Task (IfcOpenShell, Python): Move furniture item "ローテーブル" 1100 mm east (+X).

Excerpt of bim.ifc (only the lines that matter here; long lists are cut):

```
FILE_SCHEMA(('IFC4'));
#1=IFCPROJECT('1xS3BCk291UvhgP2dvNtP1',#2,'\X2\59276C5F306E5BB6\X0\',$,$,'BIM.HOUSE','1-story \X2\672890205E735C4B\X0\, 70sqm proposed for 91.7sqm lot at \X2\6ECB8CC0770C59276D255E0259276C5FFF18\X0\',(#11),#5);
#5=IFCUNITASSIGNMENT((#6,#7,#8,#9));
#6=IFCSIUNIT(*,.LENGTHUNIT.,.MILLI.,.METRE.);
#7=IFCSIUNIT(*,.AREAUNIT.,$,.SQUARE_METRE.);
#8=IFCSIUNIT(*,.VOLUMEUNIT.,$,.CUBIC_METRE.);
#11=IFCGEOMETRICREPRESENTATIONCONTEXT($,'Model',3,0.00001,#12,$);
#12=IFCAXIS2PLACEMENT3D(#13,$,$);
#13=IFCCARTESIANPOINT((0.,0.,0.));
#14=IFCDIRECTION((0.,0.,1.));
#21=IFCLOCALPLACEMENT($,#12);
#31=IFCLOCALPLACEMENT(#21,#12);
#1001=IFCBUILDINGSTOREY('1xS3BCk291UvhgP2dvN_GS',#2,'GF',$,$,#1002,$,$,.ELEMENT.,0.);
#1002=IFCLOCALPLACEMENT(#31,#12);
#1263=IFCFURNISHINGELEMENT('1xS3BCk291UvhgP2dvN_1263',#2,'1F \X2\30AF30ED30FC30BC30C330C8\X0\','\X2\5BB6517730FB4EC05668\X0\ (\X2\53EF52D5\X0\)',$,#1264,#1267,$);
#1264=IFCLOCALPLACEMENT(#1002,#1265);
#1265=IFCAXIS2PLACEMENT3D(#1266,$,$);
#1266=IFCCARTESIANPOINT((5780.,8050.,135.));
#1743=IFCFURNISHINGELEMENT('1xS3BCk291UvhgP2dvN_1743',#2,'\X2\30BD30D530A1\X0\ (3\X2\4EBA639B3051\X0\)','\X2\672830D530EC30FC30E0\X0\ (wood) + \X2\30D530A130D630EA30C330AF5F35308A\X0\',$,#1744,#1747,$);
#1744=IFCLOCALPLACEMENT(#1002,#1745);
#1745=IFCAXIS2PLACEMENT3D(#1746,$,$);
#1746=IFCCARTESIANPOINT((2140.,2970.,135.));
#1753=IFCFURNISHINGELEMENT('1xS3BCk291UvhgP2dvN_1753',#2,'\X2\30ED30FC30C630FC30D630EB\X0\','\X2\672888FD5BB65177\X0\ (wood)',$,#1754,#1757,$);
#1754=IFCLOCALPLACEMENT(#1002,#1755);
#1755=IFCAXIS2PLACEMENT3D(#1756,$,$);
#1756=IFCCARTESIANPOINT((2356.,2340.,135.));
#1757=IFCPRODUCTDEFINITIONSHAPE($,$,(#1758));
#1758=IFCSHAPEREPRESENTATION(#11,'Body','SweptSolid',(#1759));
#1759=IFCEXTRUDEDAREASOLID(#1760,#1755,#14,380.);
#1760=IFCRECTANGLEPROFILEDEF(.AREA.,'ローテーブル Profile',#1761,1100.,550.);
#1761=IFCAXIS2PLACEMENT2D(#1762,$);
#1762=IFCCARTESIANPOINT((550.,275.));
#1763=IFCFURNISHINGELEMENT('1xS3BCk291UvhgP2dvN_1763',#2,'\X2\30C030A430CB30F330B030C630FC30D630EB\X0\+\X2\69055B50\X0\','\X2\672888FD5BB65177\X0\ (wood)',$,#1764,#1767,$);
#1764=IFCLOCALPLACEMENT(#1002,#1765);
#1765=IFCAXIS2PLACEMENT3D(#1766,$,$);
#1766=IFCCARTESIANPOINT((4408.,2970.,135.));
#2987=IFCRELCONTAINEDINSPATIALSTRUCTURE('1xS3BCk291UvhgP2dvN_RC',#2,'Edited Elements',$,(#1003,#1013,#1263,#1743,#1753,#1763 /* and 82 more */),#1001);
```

```python
import ifcopenshell
import ifcopenshell.api.geometry
import ifcopenshell.util.placement
import ifcopenshell.util.unit

model = ifcopenshell.open("bim.ifc")
unit_scale = ifcopenshell.util.unit.calculate_unit_scale(model)

item = model.by_guid("1xS3BCk291UvhgP2dvN_1753")
matrix = ifcopenshell.util.placement.get_local_placement(item.ObjectPlacement)
matrix[0, 3] += 1.1 / unit_scale
ifcopenshell.api.geometry.edit_object_placement(model, product=item, matrix=matrix, is_si=False)

print(ifcopenshell.util.placement.get_local_placement(item.ObjectPlacement).round(3) + 0.0)

model.write("bim_v2.ifc")
```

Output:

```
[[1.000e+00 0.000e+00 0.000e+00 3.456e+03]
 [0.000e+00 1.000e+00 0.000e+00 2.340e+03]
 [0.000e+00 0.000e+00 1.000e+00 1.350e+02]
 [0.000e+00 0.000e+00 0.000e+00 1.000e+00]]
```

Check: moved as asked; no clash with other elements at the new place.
